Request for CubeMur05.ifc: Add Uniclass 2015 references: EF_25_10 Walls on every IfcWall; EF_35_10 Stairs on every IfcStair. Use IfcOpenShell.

First a look at what the model holds.

```python
import ifcopenshell

model = ifcopenshell.open("CubeMur05.ifc")
print(model.schema)
print("classifications:", [c.Name for c in model.by_type("IfcClassification")])
for ifc_class in ("IfcDoor", "IfcRoof", "IfcStair", "IfcWall", "IfcWindow"):
    print(ifc_class, len(model.by_type(ifc_class)))
```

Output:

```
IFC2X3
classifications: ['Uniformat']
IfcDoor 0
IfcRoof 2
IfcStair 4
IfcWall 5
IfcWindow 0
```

```python
import ifcopenshell
import ifcopenshell.api.classification

model = ifcopenshell.open("CubeMur05.ifc")

# IFC2X3 requires Source and Edition and has no link from the project to the system.
system = model.create_entity("IfcClassification", Source="NBS", Edition="2015", Name="Uniclass 2015")

codes = {
    "IfcWall": ("EF_25_10", "Walls"),
    "IfcStair": ("EF_35_10", "Stairs"),
}
for ifc_class, (code, name) in codes.items():
    products = model.by_type(ifc_class)
    ifcopenshell.api.classification.add_reference(
        model, products=products, classification=system, identification=code, name=name
    )
    print(code, len(products))

model.write("CubeMur05_updated.ifc")
```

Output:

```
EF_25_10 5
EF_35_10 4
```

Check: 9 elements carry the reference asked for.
